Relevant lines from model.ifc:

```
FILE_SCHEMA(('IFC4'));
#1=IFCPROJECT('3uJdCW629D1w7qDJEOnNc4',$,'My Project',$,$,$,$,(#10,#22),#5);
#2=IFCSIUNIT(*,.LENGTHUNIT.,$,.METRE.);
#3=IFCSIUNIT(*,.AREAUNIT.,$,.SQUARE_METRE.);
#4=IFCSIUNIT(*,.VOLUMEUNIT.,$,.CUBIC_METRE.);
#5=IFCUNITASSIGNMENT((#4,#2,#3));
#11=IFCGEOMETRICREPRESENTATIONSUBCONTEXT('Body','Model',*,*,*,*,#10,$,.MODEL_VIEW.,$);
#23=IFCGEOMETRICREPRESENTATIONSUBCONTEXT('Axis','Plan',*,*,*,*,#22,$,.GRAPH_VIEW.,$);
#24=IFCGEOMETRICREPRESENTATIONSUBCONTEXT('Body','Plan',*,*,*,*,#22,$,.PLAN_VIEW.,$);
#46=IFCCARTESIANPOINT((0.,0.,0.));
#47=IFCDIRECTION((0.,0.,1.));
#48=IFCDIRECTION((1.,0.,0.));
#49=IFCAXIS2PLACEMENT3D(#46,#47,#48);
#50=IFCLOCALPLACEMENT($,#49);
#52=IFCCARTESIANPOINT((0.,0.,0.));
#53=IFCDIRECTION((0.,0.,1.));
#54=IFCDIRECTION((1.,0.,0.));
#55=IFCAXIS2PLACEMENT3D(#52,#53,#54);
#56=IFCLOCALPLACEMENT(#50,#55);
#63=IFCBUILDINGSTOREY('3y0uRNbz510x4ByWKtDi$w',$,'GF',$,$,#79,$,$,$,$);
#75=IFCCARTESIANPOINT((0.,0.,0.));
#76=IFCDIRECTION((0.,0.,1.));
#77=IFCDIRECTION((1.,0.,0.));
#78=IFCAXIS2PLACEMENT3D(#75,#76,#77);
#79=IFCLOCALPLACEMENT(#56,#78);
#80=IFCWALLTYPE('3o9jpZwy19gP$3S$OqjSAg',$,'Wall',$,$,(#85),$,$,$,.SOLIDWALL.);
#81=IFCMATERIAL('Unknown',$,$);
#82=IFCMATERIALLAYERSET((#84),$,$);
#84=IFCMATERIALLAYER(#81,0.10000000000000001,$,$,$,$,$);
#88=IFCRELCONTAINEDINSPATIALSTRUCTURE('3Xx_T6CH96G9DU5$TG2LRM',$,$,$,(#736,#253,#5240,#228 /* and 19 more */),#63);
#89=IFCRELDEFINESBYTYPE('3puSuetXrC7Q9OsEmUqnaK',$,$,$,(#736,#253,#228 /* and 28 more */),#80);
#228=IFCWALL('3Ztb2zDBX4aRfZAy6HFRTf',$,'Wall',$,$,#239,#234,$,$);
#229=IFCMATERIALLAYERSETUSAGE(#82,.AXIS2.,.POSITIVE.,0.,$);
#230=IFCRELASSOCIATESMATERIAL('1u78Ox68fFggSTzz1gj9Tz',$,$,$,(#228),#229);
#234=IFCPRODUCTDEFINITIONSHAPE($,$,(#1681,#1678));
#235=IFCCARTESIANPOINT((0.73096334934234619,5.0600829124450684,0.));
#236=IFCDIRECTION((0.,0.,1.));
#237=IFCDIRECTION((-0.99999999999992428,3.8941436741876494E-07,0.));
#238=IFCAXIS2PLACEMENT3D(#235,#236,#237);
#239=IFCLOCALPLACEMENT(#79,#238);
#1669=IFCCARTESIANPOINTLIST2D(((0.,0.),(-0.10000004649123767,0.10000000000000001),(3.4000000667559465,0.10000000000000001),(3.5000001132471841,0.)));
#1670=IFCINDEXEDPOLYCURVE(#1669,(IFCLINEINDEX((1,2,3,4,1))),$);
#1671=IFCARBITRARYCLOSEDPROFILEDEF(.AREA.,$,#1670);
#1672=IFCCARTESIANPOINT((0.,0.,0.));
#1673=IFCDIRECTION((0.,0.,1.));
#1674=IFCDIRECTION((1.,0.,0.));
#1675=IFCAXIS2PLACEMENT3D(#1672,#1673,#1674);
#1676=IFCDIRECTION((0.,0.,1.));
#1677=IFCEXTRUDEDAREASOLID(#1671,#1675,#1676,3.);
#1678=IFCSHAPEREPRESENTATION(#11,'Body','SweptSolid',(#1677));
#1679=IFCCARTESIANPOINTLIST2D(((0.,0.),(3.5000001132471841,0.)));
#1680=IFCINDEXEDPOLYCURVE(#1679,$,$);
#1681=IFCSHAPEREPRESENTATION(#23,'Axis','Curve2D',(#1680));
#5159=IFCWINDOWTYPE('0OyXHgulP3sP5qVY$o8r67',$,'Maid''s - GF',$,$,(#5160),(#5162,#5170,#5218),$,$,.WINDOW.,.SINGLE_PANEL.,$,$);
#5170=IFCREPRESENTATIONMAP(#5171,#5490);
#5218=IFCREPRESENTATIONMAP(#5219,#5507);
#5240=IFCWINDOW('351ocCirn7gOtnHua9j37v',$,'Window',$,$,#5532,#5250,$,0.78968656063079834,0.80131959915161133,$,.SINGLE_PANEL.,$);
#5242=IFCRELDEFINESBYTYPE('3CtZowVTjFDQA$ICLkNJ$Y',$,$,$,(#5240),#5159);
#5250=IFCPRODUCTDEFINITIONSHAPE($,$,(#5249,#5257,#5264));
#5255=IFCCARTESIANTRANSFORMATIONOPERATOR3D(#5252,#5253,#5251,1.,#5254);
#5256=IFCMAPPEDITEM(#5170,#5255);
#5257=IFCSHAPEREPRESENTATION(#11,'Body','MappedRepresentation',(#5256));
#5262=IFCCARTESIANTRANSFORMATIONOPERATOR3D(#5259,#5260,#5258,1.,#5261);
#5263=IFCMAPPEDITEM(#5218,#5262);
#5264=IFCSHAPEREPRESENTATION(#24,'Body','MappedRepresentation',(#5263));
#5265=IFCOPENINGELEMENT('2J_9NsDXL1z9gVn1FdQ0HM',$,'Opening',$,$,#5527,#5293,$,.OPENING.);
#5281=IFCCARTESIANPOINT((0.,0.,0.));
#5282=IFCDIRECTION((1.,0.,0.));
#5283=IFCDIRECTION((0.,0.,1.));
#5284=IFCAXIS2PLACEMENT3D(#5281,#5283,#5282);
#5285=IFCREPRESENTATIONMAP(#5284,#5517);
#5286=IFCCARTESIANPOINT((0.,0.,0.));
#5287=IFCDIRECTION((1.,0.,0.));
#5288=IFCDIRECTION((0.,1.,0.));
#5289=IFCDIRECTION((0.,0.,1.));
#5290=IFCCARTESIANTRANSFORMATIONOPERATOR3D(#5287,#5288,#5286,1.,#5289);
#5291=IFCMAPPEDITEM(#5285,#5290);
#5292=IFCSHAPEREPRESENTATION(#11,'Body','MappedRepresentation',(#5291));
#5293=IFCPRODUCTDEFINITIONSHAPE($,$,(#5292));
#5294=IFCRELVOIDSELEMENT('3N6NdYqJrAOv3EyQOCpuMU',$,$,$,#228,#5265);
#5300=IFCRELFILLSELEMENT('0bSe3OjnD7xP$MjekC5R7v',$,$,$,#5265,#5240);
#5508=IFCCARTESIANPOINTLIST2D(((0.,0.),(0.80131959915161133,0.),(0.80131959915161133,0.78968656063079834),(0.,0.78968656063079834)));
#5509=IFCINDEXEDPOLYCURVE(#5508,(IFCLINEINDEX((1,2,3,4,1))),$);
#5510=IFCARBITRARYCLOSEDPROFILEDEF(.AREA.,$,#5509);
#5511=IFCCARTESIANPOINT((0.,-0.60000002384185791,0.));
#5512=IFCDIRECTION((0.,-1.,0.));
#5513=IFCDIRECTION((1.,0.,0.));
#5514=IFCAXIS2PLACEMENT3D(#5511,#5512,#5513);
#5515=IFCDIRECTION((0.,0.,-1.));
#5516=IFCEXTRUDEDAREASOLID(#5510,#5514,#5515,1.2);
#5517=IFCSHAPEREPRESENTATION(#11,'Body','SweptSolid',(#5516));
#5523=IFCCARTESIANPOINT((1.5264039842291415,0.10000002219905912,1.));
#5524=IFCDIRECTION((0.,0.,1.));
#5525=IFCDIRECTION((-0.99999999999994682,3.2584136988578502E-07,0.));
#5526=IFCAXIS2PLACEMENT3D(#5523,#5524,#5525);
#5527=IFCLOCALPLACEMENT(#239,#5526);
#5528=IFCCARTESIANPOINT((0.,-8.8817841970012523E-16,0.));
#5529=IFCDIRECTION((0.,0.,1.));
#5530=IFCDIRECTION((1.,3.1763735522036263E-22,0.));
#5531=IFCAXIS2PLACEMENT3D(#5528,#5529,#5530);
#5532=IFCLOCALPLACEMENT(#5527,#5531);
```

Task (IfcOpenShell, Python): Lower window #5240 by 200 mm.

```python
import numpy as np
import ifcopenshell
import ifcopenshell.api.geometry
import ifcopenshell.util.placement
import ifcopenshell.util.unit

model = ifcopenshell.open("model.ifc")
unit_scale = ifcopenshell.util.unit.calculate_unit_scale(model)

window = model.by_guid("351ocCirn7gOtnHua9j37v")
opening = window.FillsVoids[0].RelatingOpeningElement
dz = -0.2 / unit_scale

shift = np.array([0.0, 0.0, dz])
# The window is placed relative to its opening, so it follows when the opening moves.
matrix = ifcopenshell.util.placement.get_local_placement(opening.ObjectPlacement)
matrix[:3, 3] += shift
ifcopenshell.api.geometry.edit_object_placement(
    model, product=opening, matrix=matrix, is_si=False, should_transform_children=True
)

print(f"moved by {dz * unit_scale:+.3f} m")

model.write("model_v2.ifc")
```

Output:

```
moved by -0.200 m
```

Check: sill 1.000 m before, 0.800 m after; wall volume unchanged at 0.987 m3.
